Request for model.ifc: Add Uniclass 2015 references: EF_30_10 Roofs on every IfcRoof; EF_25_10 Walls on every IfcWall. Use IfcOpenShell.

First a look at what the model holds.

```python
import ifcopenshell

model = ifcopenshell.open("model.ifc")
print(model.schema)
print("classifications:", [c.Name for c in model.by_type("IfcClassification")])
for ifc_class in ("IfcDoor", "IfcRoof", "IfcStair", "IfcWall", "IfcWindow"):
    print(ifc_class, len(model.by_type(ifc_class)))
```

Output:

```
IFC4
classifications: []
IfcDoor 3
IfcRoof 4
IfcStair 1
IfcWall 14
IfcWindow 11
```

```python
import ifcopenshell
import ifcopenshell.api.classification

model = ifcopenshell.open("model.ifc")

system = ifcopenshell.api.classification.add_classification(model, classification="Uniclass 2015")

codes = {
    "IfcRoof": ("EF_30_10", "Roofs"),
    "IfcWall": ("EF_25_10", "Walls"),
}
for ifc_class, (code, name) in codes.items():
    products = model.by_type(ifc_class)
    ifcopenshell.api.classification.add_reference(
        model, products=products, classification=system, identification=code, name=name
    )
    print(code, len(products))

model.write("model_rev.ifc")
```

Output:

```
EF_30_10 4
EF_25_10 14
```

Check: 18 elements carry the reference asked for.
